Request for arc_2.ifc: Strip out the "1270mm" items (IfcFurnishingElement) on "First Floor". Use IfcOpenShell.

First a look at what the model holds.

```python
import ifcopenshell
import ifcopenshell.util.element

model = ifcopenshell.open("arc_2.ifc")
print(model.schema)
storey = next(s for s in model.by_type("IfcBuildingStorey") if s.Name == "First Floor")
furniture = [e for e in ifcopenshell.util.element.get_decomposition(storey) if e.is_a("IfcFurnishingElement")]
seen = {}
for e in furniture:
    element_type = ifcopenshell.util.element.get_type(e)
    name = element_type.Name if element_type not in (None, e) else None
    seen[name] = seen.get(name, 0) + 1
for name, count in sorted(seen.items(), key=str):
    print(count, "x", name)
```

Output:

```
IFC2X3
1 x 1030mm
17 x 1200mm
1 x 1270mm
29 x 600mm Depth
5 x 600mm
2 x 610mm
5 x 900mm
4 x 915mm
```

```python
import ifcopenshell
import ifcopenshell.api.root
import ifcopenshell.util.element

model = ifcopenshell.open("arc_2.ifc")

storey = next(s for s in model.by_type("IfcBuildingStorey") if s.Name == "First Floor")
furniture = [e for e in ifcopenshell.util.element.get_decomposition(storey) if e.is_a("IfcFurnishingElement")]
targets = [e for e in furniture if (t := ifcopenshell.util.element.get_type(e)) not in (None, e) and t.Name == "1270mm"]

for e in targets:
    ifcopenshell.api.root.remove_product(model, product=e)
print(len(targets), "removed")

model.write("arc_2_v2.ifc")
```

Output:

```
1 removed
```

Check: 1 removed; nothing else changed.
